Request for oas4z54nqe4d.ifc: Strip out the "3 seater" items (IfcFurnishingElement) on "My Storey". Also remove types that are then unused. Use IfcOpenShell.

First a look at what the model holds.

```python
import ifcopenshell
import ifcopenshell.util.element

model = ifcopenshell.open("oas4z54nqe4d.ifc")
print(model.schema)
storey = next(s for s in model.by_type("IfcBuildingStorey") if s.Name == "My Storey")
furniture = [e for e in ifcopenshell.util.element.get_decomposition(storey) if e.is_a("IfcFurnishingElement")]
seen = {}
for e in furniture:
    element_type = ifcopenshell.util.element.get_type(e)
    name = element_type.Name if element_type not in (None, e) else None
    seen[name] = seen.get(name, 0) + 1
for name, count in sorted(seen.items(), key=str):
    print(count, "x", name)
```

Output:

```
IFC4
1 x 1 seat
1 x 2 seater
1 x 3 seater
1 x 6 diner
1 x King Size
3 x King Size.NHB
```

```python
import ifcopenshell
import ifcopenshell.api.root
import ifcopenshell.util.element

model = ifcopenshell.open("oas4z54nqe4d.ifc")

storey = next(s for s in model.by_type("IfcBuildingStorey") if s.Name == "My Storey")
furniture = [e for e in ifcopenshell.util.element.get_decomposition(storey) if e.is_a("IfcFurnishingElement")]
targets = [e for e in furniture if (t := ifcopenshell.util.element.get_type(e)) not in (None, e) and t.Name == "3 seater"]
types = {ifcopenshell.util.element.get_type(e) for e in targets} - {None, *targets}

for e in targets:
    ifcopenshell.api.root.remove_product(model, product=e)
print(len(targets), "removed")

unused = [t for t in types if not ifcopenshell.util.element.get_types(t)]
for t in unused:
    ifcopenshell.api.root.remove_product(model, product=t)
print(len(unused), "unused types removed")

model.write("oas4z54nqe4d_edited.ifc")
```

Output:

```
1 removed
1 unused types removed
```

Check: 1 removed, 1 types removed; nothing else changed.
